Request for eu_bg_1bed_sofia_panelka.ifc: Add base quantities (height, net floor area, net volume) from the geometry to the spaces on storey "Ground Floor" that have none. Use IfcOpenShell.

First a look at what the model holds.

```python
import ifcopenshell
import ifcopenshell.util.element
import ifcopenshell.util.unit

model = ifcopenshell.open("eu_bg_1bed_sofia_panelka.ifc")
print(model.schema)
for unit_type in ("LENGTHUNIT", "AREAUNIT", "VOLUMEUNIT"):
    print(unit_type, ifcopenshell.util.unit.calculate_unit_scale(model, unit_type))
storey = next(s for s in model.by_type("IfcBuildingStorey") if s.Name == "Ground Floor")
spaces = [e for e in ifcopenshell.util.element.get_decomposition(storey) if e.is_a("IfcSpace")]
for e in sorted(spaces, key=lambda e: e.id()):
    print(e.id(), e.is_a(), e.Name, list(ifcopenshell.util.element.get_psets(e, qtos_only=True)), sep=" | ")
```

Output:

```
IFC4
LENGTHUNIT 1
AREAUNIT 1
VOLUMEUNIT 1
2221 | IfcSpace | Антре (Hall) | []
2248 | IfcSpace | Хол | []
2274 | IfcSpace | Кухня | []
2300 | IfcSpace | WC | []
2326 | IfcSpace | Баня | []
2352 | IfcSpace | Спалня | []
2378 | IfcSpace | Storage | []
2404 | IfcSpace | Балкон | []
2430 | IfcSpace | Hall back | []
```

```python
import ifcopenshell
import ifcopenshell.api.pset
import ifcopenshell.geom
import ifcopenshell.util.element
import ifcopenshell.util.shape
import ifcopenshell.util.unit

model = ifcopenshell.open("eu_bg_1bed_sofia_panelka.ifc")
unit_scale = ifcopenshell.util.unit.calculate_unit_scale(model)
area_scale = ifcopenshell.util.unit.calculate_unit_scale(model, "AREAUNIT")
volume_scale = ifcopenshell.util.unit.calculate_unit_scale(model, "VOLUMEUNIT")
settings = ifcopenshell.geom.settings()

storey = next(s for s in model.by_type("IfcBuildingStorey") if s.Name == "Ground Floor")
spaces = [e for e in ifcopenshell.util.element.get_decomposition(storey) if e.is_a("IfcSpace")]

for e in sorted(spaces, key=lambda e: e.id()):
    if ifcopenshell.util.element.get_psets(e, qtos_only=True, should_inherit=False):
        continue
    # Geometry comes back in metres, in the element's own axes.
    shape = ifcopenshell.geom.create_shape(settings, e)
    values = {
        "Height": ifcopenshell.util.shape.get_z(shape.geometry) / unit_scale,
        "NetFloorArea": ifcopenshell.util.shape.get_footprint_area(shape.geometry) / area_scale,
        "NetVolume": ifcopenshell.util.shape.get_volume(shape.geometry) / volume_scale,
    }
    qto = ifcopenshell.api.pset.add_qto(model, product=e, name="Qto_SpaceBaseQuantities")
    ifcopenshell.api.pset.edit_qto(model, qto=qto, properties=values)
    print(e.id(), {k: round(v, 3) for k, v in values.items()})

model.write("eu_bg_1bed_sofia_panelka_v2.ifc")
```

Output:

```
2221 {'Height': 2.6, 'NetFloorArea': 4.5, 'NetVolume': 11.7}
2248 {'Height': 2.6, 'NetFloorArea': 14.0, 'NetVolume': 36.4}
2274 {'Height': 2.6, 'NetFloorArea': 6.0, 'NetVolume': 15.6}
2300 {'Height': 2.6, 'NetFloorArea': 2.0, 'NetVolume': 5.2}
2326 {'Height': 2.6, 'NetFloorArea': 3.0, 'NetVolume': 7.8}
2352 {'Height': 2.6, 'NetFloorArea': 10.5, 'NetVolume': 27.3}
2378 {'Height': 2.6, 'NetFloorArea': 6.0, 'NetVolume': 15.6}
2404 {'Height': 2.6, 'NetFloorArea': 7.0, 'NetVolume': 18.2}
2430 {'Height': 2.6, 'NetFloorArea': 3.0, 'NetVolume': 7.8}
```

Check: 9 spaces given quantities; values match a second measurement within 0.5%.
